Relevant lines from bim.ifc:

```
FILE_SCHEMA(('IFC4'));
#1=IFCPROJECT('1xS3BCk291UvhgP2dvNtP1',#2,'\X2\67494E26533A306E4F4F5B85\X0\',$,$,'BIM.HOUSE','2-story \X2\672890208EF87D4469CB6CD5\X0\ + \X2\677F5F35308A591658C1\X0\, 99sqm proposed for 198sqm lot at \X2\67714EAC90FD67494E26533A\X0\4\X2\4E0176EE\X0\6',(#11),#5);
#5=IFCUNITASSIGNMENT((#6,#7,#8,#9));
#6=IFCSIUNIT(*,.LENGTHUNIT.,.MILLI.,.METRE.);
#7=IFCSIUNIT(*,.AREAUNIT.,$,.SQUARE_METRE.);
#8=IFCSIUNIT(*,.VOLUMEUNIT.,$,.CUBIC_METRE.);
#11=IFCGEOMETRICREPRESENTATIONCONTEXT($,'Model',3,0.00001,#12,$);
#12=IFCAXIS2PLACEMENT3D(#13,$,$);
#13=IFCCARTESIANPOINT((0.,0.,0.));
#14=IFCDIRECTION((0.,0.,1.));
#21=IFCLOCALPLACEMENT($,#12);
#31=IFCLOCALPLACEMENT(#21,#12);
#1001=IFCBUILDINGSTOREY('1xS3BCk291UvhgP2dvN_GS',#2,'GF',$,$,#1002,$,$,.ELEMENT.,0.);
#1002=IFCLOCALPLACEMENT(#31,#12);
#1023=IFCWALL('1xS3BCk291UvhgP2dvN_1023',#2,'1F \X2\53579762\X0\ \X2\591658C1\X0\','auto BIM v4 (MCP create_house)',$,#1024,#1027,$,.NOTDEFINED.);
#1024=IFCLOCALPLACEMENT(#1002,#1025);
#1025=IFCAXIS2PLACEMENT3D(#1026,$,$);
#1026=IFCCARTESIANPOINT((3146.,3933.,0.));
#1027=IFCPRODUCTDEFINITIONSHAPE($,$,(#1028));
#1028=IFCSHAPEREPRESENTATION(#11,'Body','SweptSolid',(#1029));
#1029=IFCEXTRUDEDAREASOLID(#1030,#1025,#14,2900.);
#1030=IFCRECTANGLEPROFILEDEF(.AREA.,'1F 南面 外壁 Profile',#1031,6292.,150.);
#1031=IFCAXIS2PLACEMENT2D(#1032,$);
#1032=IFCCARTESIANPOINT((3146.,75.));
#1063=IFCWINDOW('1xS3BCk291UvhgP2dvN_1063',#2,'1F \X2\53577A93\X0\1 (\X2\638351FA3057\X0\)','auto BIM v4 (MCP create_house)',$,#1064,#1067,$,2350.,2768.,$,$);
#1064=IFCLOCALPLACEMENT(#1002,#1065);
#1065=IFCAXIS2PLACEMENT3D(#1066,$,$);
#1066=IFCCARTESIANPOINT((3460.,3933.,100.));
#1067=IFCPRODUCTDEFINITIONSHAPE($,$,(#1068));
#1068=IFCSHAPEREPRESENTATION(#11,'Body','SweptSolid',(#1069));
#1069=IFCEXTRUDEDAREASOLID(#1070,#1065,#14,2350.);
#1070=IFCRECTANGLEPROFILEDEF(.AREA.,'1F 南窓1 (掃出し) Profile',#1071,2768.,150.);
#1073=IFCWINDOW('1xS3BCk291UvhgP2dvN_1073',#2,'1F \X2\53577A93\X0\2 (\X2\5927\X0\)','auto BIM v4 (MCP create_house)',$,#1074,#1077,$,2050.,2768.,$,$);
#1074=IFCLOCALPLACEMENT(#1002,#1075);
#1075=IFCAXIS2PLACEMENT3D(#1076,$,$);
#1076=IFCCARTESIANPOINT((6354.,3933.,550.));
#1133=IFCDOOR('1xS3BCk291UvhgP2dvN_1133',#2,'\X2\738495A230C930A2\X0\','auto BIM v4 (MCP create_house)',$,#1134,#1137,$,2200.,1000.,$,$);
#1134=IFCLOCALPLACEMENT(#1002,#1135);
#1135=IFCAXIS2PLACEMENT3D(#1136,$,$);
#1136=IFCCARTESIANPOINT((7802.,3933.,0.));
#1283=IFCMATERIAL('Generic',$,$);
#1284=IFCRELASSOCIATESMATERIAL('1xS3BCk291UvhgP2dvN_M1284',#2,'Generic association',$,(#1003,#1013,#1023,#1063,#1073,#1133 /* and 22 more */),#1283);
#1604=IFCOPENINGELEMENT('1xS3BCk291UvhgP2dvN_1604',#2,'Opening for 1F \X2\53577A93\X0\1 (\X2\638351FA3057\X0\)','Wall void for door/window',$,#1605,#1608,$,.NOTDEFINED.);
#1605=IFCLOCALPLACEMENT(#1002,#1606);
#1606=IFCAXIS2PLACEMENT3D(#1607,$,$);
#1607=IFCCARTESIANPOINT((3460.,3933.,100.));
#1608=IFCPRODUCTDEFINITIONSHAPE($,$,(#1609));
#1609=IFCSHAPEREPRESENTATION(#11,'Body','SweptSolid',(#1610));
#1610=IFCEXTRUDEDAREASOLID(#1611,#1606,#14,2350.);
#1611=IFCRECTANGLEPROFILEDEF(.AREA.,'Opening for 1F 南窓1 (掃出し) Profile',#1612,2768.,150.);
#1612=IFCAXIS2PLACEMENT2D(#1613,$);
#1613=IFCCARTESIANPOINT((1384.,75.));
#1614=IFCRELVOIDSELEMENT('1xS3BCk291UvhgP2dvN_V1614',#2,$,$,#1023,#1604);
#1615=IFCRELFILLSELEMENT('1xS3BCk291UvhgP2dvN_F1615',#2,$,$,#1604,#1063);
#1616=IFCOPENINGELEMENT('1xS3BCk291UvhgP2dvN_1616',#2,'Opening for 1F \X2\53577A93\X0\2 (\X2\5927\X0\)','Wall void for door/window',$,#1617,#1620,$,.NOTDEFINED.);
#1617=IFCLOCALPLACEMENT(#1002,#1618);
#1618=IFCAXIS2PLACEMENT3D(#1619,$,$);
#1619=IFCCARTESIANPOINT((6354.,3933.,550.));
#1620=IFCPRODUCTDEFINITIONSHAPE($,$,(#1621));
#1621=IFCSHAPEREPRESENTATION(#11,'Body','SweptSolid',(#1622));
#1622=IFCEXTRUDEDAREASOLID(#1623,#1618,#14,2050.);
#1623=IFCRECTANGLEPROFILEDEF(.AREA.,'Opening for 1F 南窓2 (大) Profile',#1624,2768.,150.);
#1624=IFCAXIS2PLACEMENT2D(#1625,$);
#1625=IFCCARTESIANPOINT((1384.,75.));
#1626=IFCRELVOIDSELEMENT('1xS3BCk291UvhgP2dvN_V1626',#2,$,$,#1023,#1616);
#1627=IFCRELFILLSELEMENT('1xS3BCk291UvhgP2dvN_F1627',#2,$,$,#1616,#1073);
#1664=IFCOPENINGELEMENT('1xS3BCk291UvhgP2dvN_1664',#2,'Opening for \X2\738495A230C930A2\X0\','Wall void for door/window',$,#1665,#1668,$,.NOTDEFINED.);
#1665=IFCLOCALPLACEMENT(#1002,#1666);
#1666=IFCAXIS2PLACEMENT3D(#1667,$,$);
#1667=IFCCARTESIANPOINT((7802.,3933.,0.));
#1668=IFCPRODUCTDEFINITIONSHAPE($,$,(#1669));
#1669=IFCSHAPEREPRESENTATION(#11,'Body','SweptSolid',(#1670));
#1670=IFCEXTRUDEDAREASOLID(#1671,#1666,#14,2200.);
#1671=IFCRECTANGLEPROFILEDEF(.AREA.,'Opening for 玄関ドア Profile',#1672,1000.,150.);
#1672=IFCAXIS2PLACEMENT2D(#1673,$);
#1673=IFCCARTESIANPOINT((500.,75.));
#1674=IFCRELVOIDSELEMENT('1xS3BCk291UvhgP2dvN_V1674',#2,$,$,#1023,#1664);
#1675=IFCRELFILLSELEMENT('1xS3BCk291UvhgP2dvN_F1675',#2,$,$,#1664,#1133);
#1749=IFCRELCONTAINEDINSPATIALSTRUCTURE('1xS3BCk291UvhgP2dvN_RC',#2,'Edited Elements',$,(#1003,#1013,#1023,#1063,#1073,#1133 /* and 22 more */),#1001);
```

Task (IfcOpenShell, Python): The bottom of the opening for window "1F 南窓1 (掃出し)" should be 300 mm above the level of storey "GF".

```python
import numpy as np
import ifcopenshell
import ifcopenshell.api.geometry
import ifcopenshell.geom
import ifcopenshell.util.element
import ifcopenshell.util.placement
import ifcopenshell.util.shape
import ifcopenshell.util.unit

model = ifcopenshell.open("bim.ifc")
unit_scale = ifcopenshell.util.unit.calculate_unit_scale(model)

window = model.by_guid("1xS3BCk291UvhgP2dvN_1063")
opening = window.FillsVoids[0].RelatingOpeningElement
storey = ifcopenshell.util.element.get_container(window, ifc_class="IfcBuildingStorey")
level = ifcopenshell.util.placement.get_local_placement(storey.ObjectPlacement)[2, 3]

# The opening's origin need not be at the sill, so measure its lowest point.
shape = ifcopenshell.geom.create_shape(ifcopenshell.geom.settings(), opening)
bottom = ifcopenshell.util.shape.get_shape_bottom_elevation(shape, shape.geometry) / unit_scale
dz = level + 0.3 / unit_scale - bottom

shift = np.array([0.0, 0.0, dz])
# The window is not placed relative to its opening, so move both.
for product in (opening, window):
    matrix = ifcopenshell.util.placement.get_local_placement(product.ObjectPlacement)
    matrix[:3, 3] += shift
    ifcopenshell.api.geometry.edit_object_placement(model, product=product, matrix=matrix, is_si=False)

print(f"moved by {dz * unit_scale:+.3f} m")

model.write("bim-out.ifc")
```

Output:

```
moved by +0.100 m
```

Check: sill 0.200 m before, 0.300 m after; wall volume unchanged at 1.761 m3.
